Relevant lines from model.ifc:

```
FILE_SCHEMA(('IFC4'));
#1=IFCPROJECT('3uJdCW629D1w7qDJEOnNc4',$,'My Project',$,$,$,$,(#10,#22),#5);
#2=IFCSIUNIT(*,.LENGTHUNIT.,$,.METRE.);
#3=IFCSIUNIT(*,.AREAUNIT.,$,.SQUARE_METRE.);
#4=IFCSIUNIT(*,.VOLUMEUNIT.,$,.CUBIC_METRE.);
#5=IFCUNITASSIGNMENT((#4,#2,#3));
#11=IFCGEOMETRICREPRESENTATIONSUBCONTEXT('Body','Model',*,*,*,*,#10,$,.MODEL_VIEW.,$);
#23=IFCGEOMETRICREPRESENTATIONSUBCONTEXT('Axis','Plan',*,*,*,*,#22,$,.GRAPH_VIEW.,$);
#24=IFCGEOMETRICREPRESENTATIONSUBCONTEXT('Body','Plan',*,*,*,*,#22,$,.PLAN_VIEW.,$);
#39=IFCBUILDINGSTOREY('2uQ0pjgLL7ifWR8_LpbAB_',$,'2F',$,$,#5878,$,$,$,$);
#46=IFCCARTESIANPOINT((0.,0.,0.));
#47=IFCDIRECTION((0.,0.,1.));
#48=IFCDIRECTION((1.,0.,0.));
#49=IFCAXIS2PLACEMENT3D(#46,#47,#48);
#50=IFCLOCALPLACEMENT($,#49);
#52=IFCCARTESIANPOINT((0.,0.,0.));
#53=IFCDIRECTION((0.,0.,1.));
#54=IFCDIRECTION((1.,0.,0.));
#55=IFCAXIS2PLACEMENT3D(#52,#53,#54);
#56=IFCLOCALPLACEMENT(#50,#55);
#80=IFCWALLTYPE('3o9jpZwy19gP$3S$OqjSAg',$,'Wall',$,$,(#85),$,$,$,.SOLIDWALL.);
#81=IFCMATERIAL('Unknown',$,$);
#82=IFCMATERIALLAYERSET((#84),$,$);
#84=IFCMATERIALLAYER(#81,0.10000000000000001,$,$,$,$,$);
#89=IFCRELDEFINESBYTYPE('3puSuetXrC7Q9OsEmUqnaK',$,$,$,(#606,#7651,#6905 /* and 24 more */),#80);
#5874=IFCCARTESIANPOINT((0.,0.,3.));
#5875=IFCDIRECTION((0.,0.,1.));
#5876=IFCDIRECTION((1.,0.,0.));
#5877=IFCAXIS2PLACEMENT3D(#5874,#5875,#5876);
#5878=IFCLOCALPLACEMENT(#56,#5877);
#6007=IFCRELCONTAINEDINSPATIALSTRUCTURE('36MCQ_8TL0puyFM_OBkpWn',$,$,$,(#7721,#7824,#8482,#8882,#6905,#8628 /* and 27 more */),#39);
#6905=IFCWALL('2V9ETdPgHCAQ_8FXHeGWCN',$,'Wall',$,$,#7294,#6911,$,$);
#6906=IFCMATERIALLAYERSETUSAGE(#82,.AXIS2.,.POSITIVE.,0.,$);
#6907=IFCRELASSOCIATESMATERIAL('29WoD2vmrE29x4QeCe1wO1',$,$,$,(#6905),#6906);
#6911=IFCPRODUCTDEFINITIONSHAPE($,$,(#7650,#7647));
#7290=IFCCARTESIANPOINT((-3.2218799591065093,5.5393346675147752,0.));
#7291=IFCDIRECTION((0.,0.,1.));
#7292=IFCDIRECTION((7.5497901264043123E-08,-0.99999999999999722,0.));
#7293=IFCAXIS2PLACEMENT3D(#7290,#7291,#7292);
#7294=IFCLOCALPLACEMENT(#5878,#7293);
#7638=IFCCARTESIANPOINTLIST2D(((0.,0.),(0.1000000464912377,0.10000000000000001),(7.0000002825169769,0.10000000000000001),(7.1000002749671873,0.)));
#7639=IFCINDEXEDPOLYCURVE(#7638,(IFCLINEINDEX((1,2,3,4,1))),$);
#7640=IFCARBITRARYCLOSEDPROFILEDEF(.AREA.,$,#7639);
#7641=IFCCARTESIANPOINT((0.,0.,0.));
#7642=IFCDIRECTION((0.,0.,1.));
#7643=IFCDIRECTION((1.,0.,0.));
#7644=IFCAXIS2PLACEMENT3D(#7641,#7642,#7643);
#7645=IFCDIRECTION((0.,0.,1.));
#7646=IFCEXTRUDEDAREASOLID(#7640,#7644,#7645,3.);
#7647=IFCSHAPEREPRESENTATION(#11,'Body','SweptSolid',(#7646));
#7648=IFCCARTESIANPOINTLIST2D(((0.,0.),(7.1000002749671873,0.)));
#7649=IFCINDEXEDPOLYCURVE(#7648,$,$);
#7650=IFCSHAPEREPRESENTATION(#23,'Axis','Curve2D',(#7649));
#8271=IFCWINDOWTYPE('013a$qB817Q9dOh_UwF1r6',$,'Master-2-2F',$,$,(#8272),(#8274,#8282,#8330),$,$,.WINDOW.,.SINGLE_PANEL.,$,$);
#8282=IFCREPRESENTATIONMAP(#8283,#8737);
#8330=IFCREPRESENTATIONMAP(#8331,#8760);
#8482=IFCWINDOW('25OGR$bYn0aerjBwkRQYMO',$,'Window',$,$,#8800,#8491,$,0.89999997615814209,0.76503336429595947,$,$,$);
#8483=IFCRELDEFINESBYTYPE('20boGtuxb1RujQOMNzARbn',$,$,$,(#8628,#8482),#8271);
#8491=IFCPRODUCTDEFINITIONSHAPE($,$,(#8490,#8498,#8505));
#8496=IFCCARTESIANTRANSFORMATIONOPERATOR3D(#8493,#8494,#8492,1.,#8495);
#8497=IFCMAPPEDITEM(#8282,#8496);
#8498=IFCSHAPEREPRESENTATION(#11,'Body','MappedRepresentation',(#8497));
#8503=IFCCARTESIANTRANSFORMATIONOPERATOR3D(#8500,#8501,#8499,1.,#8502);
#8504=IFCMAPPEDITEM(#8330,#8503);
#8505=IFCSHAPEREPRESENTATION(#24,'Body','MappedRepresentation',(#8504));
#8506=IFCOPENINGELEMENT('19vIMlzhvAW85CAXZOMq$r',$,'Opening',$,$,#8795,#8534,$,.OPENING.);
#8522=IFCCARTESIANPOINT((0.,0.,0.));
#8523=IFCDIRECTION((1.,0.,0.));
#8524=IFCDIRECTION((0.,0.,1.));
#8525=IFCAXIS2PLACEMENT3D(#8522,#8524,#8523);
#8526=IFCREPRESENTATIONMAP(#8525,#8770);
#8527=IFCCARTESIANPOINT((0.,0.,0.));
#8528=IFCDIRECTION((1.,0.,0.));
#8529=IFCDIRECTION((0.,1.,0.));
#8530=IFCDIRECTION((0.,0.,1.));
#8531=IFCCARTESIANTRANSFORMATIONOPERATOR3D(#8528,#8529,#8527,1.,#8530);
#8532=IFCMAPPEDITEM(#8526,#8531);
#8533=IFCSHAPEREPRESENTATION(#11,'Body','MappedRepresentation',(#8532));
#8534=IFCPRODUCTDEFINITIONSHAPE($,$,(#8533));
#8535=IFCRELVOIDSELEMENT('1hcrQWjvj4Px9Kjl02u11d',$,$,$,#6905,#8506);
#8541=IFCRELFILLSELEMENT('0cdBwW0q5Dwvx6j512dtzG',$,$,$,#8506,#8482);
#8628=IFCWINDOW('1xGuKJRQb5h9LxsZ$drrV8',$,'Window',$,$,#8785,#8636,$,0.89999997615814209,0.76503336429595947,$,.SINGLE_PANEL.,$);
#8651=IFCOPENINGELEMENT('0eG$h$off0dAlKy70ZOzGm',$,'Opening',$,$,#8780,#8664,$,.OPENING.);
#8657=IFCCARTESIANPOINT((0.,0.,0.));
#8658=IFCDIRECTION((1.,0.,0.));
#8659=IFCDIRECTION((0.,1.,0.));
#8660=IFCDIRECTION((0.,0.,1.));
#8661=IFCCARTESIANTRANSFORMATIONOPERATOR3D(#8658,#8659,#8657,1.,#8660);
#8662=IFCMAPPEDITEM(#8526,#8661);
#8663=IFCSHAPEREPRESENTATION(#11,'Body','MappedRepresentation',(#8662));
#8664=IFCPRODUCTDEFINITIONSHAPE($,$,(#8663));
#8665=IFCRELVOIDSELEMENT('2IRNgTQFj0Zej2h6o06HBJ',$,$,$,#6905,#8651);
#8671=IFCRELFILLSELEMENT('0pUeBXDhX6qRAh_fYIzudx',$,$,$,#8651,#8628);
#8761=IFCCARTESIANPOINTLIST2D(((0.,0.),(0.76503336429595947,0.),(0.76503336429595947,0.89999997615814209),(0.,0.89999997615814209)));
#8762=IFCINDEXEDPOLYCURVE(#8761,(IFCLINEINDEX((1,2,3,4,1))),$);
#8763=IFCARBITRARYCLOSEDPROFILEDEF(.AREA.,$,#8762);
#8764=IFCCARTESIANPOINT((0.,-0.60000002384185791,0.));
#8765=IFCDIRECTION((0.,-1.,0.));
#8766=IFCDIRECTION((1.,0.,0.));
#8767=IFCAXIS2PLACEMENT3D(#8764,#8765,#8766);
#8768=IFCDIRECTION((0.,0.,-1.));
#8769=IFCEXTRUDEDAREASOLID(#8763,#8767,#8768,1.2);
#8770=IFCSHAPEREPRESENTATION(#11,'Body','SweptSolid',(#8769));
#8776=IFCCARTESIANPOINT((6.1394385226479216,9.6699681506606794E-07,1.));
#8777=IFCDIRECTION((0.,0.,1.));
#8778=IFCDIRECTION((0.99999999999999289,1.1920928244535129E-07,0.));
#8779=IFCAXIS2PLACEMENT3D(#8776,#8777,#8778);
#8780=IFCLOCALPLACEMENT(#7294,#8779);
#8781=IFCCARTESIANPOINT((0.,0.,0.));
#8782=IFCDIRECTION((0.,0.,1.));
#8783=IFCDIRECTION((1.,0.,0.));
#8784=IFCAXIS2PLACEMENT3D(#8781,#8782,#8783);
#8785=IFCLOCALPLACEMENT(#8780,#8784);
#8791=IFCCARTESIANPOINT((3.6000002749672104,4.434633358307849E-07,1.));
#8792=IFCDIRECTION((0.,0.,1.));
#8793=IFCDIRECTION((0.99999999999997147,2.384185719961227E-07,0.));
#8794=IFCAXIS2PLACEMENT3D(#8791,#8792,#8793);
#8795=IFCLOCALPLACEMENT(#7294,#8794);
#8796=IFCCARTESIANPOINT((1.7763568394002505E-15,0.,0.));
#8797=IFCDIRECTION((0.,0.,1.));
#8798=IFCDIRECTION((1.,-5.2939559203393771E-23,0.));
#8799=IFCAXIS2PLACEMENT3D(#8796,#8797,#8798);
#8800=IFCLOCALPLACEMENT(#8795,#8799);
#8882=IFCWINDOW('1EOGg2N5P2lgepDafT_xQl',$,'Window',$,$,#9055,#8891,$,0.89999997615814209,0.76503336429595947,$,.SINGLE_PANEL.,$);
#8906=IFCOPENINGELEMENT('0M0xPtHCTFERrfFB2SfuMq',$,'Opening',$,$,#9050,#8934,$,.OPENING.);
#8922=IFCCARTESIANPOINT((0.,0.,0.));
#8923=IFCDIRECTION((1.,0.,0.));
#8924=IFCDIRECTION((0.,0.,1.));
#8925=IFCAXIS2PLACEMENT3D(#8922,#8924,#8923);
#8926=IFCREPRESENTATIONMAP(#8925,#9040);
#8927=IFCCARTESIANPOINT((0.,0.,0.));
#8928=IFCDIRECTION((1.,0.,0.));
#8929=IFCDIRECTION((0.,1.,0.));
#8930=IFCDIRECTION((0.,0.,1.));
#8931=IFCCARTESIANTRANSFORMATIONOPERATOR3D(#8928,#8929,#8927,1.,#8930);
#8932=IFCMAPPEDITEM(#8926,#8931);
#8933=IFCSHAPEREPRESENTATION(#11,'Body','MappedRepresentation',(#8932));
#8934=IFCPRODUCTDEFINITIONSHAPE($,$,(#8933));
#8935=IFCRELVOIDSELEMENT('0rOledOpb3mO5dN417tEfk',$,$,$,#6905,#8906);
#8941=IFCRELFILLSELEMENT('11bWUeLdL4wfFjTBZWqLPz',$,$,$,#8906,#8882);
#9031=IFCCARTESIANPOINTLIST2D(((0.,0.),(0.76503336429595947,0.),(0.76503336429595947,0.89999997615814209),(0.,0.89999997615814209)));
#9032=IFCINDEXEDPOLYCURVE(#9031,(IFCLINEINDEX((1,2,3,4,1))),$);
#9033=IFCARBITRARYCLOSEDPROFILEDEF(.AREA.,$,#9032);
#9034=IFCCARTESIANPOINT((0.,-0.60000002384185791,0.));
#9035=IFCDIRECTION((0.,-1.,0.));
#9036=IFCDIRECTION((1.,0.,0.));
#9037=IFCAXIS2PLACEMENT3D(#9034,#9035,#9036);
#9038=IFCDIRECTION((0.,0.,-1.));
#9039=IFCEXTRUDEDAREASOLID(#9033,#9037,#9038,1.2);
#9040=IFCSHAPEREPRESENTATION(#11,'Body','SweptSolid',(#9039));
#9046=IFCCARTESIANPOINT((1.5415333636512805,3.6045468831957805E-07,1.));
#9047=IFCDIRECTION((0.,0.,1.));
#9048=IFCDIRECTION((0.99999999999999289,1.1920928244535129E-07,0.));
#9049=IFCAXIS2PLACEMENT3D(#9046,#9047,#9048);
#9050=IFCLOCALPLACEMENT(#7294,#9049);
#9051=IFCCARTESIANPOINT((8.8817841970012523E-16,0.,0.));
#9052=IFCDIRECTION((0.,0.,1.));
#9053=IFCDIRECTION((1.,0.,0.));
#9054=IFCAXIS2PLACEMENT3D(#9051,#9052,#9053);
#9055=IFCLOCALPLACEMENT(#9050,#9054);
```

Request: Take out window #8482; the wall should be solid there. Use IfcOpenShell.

```python
import ifcopenshell
import ifcopenshell.api.feature
import ifcopenshell.api.root
import ifcopenshell.geom
import ifcopenshell.util.shape

model = ifcopenshell.open("model.ifc")
settings = ifcopenshell.geom.settings()


def volume(element):
    """Net volume in cubic metres, openings subtracted."""
    shape = ifcopenshell.geom.create_shape(settings, element)
    return ifcopenshell.util.shape.get_volume(shape.geometry)


window = model.by_guid("25OGR$bYn0aerjBwkRQYMO")
opening = window.FillsVoids[0].RelatingOpeningElement
wall = opening.VoidsElements[0].RelatingBuildingElement
before = volume(wall)

ifcopenshell.api.root.remove_product(model, product=window)
ifcopenshell.api.feature.remove_feature(model, feature=opening)

after = volume(wall)

print(f"wall volume {before:.3f} -> {after:.3f} m3")

model.write("model-out.ifc")
```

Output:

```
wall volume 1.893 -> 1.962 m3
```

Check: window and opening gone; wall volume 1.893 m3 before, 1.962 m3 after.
